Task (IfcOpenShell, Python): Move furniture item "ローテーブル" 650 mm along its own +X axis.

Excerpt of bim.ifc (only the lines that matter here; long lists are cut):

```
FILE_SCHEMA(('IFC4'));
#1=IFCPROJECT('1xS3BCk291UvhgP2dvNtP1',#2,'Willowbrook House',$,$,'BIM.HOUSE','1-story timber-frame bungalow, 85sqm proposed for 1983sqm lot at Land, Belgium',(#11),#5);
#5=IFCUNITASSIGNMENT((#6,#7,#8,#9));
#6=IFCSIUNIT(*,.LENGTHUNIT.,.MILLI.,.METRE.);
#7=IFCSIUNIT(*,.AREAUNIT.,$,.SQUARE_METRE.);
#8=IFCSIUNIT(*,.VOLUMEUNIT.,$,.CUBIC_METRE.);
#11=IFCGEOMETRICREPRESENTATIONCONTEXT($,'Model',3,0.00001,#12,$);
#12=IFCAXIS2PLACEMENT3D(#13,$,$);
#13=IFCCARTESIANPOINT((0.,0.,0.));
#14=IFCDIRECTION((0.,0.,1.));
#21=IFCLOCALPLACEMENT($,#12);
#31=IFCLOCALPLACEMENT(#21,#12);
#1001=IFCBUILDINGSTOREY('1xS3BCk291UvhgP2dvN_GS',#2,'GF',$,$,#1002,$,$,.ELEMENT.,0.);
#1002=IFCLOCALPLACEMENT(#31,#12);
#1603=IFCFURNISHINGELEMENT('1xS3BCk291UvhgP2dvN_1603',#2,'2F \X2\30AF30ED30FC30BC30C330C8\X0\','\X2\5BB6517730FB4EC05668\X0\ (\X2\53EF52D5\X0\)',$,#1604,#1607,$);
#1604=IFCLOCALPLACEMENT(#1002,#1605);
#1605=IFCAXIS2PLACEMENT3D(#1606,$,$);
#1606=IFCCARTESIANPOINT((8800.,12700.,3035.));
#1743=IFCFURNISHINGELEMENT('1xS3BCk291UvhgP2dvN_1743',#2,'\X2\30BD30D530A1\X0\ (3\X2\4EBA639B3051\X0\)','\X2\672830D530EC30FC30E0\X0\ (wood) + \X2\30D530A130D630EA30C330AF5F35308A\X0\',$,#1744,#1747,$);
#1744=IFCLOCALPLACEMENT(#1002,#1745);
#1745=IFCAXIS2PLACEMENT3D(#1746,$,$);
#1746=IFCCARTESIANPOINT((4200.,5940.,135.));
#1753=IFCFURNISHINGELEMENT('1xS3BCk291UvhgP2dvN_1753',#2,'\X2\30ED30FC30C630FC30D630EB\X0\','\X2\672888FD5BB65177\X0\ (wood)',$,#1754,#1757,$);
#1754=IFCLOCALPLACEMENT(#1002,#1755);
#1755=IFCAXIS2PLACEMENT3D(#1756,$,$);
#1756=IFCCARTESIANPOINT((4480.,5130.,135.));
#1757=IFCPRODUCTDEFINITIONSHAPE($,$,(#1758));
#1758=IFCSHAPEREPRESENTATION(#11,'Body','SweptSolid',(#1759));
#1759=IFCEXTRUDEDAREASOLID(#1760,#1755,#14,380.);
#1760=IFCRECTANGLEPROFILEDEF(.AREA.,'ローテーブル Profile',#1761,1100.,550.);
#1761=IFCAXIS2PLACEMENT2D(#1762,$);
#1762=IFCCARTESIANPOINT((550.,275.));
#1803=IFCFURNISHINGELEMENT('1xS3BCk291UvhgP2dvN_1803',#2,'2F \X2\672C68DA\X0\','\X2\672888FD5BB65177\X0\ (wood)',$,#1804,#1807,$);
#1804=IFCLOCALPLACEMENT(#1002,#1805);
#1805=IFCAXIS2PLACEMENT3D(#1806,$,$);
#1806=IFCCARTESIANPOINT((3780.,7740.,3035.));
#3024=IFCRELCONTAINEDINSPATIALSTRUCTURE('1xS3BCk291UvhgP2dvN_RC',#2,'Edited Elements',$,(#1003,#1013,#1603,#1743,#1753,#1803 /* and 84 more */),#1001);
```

```python
import ifcopenshell
import ifcopenshell.api.geometry
import ifcopenshell.util.placement
import ifcopenshell.util.unit

model = ifcopenshell.open("bim.ifc")
unit_scale = ifcopenshell.util.unit.calculate_unit_scale(model)

item = model.by_id(1753)
matrix = ifcopenshell.util.placement.get_local_placement(item.ObjectPlacement)
matrix[:3, 3] += matrix[:3, 0] * 0.65 / unit_scale
ifcopenshell.api.geometry.edit_object_placement(model, product=item, matrix=matrix, is_si=False)

print(ifcopenshell.util.placement.get_local_placement(item.ObjectPlacement).round(3) + 0.0)

model.write("bim_updated.ifc")
```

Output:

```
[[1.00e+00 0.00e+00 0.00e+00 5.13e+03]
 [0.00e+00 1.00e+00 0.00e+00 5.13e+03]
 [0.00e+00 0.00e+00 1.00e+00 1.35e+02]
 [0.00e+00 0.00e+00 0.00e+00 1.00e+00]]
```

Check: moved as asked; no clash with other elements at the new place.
